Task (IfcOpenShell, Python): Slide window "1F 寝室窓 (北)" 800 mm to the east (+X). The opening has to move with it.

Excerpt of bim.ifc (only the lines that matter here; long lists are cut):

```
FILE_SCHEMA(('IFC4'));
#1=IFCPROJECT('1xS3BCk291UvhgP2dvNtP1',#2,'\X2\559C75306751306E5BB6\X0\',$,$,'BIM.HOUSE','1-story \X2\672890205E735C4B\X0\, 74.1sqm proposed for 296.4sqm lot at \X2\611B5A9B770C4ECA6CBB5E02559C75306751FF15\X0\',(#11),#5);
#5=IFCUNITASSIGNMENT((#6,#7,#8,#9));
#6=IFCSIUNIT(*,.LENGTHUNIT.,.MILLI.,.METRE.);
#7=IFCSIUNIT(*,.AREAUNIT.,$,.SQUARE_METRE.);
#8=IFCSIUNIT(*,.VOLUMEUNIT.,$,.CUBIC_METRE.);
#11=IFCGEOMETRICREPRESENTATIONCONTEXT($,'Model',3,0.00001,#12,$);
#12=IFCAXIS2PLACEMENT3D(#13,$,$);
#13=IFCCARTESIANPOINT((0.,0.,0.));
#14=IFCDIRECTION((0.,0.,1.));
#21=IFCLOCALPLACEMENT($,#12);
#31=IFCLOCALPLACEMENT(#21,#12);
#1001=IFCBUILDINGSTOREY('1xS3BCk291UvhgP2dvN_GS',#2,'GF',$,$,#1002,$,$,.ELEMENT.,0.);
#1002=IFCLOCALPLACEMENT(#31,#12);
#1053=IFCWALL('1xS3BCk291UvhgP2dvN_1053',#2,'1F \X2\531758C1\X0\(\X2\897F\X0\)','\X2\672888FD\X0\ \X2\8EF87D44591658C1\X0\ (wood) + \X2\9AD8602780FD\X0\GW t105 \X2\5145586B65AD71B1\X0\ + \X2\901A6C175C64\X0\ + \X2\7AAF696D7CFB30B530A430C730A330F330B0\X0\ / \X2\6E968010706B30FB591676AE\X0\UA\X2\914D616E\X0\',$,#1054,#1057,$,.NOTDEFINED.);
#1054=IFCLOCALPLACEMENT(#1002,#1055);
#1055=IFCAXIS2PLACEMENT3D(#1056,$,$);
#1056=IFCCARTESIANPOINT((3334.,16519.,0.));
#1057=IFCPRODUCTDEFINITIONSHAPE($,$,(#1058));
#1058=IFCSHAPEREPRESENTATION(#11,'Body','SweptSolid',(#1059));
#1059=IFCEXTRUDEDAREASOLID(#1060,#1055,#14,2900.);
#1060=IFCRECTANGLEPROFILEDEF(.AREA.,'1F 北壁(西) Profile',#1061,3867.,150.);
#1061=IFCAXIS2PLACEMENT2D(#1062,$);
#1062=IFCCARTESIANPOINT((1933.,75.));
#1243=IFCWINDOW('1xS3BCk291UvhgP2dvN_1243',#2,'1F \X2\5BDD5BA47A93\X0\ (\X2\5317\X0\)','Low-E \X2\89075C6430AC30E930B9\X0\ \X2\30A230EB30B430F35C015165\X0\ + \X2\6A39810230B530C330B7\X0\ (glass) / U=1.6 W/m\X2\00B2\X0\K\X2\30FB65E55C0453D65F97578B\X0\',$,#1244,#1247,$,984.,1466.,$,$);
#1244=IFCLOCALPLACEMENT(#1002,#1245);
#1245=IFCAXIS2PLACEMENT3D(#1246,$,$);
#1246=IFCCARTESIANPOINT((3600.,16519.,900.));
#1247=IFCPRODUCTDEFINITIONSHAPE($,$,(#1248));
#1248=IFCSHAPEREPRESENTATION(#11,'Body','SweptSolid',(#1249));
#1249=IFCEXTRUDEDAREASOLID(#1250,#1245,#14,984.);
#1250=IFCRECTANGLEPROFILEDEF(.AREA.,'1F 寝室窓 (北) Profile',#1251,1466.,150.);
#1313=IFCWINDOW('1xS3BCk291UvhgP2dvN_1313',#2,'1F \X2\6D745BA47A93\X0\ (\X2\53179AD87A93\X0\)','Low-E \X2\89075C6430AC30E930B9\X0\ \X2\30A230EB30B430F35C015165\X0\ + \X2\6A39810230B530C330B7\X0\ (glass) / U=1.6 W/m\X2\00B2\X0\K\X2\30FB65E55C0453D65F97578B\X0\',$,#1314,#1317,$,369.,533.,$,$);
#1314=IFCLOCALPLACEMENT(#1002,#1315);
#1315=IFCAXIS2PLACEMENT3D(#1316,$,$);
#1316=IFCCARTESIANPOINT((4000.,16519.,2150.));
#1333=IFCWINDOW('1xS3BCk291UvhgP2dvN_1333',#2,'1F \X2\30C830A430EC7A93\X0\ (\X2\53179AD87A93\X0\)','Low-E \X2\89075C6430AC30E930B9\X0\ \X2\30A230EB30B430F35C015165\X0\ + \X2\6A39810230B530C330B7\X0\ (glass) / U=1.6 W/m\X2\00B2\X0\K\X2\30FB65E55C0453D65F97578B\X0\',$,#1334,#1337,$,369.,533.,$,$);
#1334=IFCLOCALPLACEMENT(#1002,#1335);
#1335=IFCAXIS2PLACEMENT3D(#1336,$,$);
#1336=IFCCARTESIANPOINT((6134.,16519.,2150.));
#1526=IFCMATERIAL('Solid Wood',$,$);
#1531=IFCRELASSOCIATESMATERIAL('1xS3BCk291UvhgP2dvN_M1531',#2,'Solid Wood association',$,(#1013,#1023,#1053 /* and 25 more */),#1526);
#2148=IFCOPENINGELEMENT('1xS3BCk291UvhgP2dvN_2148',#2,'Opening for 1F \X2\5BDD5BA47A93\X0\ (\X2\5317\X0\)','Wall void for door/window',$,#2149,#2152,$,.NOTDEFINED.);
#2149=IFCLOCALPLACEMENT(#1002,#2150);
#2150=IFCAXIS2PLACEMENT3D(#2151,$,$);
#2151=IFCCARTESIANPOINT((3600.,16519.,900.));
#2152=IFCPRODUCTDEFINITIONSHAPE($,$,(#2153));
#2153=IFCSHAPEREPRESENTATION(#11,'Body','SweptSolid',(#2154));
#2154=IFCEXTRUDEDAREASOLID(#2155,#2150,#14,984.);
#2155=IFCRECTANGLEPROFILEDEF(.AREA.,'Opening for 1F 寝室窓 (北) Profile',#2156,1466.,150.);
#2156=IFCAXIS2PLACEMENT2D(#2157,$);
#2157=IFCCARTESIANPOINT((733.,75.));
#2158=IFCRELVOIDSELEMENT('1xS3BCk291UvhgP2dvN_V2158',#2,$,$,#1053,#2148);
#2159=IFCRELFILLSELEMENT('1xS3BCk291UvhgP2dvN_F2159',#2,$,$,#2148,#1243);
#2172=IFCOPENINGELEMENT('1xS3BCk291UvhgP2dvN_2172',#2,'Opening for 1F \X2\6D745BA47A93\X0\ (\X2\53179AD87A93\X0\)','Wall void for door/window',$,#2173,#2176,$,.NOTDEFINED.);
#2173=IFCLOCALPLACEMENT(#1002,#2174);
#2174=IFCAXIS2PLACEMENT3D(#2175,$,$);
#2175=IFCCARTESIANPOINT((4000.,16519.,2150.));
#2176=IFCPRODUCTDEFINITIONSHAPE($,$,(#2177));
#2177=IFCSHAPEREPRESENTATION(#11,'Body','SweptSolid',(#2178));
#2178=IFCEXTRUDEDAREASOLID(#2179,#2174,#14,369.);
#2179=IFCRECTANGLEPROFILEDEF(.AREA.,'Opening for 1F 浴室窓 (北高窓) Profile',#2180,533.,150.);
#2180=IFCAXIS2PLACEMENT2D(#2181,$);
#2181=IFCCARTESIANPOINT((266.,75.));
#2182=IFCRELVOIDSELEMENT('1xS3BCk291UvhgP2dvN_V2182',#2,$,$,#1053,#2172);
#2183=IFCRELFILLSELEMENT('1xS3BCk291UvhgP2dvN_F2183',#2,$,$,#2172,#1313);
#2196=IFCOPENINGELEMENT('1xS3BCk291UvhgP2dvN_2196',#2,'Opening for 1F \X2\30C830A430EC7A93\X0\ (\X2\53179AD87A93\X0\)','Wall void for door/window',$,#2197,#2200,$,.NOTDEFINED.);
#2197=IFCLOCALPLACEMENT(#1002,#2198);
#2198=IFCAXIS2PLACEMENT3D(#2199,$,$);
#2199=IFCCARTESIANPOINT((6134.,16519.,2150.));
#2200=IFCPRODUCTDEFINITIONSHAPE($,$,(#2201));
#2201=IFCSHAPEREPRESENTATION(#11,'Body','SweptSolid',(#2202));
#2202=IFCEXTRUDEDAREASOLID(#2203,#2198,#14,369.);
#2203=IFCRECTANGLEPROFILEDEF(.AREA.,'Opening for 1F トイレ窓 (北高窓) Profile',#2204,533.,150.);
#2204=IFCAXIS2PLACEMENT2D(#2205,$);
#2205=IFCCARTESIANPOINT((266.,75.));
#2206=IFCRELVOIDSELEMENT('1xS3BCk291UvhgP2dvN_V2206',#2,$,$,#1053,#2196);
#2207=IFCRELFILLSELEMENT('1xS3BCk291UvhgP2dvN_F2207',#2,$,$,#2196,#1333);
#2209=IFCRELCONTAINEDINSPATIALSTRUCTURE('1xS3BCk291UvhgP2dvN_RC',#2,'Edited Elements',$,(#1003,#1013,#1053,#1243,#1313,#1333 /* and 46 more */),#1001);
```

```python
import ifcopenshell
import ifcopenshell.api.geometry
import ifcopenshell.util.placement
import ifcopenshell.util.unit

model = ifcopenshell.open("bim.ifc")
unit_scale = ifcopenshell.util.unit.calculate_unit_scale(model)

window = model.by_guid("1xS3BCk291UvhgP2dvN_1243")
opening = window.FillsVoids[0].RelatingOpeningElement
wall = opening.VoidsElements[0].RelatingBuildingElement

wall_matrix = ifcopenshell.util.placement.get_local_placement(wall.ObjectPlacement)
shift = wall_matrix[:3, 0] * 0.8 / unit_scale
before = ifcopenshell.util.placement.get_local_placement(window.ObjectPlacement)[:3, 3].copy()

# The window is not placed relative to its opening, so move both.
for product in (opening, window):
    matrix = ifcopenshell.util.placement.get_local_placement(product.ObjectPlacement)
    matrix[:3, 3] += shift
    ifcopenshell.api.geometry.edit_object_placement(model, product=product, matrix=matrix, is_si=False)

after = ifcopenshell.util.placement.get_local_placement(window.ObjectPlacement)[:3, 3]
print("window moved by", (after - before).round(3) + 0.0)

model.write("bim_rev.ifc")
```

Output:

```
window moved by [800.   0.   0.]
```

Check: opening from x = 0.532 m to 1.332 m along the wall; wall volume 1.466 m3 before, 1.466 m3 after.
